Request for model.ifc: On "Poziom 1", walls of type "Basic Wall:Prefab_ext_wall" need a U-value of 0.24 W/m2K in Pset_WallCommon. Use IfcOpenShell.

First a look at what the model holds.

```python
import ifcopenshell
import ifcopenshell.util.element

model = ifcopenshell.open("model.ifc")
print(model.schema)
storey = next(s for s in model.by_type("IfcBuildingStorey") if s.Name == "Poziom 1")
walls = [e for e in ifcopenshell.util.element.get_decomposition(storey) if e.is_a("IfcWall")]
seen = {}
for e in walls:
    element_type = ifcopenshell.util.element.get_type(e)
    key = (element_type.Name if element_type != e and element_type else None, ifcopenshell.util.element.get_pset(e, "Pset_WallCommon", "ThermalTransmittance"))
    seen[key] = seen.get(key, 0) + 1
for (name, value), count in sorted(seen.items(), key=str):
    print(count, "x", name, "|", value)
```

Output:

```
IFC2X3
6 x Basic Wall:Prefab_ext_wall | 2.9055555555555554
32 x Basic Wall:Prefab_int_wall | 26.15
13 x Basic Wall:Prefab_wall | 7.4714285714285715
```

```python
import ifcopenshell
import ifcopenshell.api.pset
import ifcopenshell.util.element

model = ifcopenshell.open("model.ifc")

storey = next(s for s in model.by_type("IfcBuildingStorey") if s.Name == "Poziom 1")
walls = [e for e in ifcopenshell.util.element.get_decomposition(storey) if e.is_a("IfcWall")]

count = 0
for e in walls:
    element_type = ifcopenshell.util.element.get_type(e)
    if element_type in (None, e) or element_type.Name != "Basic Wall:Prefab_ext_wall":
        continue
    # add_pset returns the element's existing set when there is one.
    pset = ifcopenshell.api.pset.add_pset(model, product=e, name="Pset_WallCommon")
    ifcopenshell.api.pset.edit_pset(model, pset=pset, properties={"ThermalTransmittance": 0.24})
    count += 1

print(count, "walls updated")

model.write("model_updated.ifc")
```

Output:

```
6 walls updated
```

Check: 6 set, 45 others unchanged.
